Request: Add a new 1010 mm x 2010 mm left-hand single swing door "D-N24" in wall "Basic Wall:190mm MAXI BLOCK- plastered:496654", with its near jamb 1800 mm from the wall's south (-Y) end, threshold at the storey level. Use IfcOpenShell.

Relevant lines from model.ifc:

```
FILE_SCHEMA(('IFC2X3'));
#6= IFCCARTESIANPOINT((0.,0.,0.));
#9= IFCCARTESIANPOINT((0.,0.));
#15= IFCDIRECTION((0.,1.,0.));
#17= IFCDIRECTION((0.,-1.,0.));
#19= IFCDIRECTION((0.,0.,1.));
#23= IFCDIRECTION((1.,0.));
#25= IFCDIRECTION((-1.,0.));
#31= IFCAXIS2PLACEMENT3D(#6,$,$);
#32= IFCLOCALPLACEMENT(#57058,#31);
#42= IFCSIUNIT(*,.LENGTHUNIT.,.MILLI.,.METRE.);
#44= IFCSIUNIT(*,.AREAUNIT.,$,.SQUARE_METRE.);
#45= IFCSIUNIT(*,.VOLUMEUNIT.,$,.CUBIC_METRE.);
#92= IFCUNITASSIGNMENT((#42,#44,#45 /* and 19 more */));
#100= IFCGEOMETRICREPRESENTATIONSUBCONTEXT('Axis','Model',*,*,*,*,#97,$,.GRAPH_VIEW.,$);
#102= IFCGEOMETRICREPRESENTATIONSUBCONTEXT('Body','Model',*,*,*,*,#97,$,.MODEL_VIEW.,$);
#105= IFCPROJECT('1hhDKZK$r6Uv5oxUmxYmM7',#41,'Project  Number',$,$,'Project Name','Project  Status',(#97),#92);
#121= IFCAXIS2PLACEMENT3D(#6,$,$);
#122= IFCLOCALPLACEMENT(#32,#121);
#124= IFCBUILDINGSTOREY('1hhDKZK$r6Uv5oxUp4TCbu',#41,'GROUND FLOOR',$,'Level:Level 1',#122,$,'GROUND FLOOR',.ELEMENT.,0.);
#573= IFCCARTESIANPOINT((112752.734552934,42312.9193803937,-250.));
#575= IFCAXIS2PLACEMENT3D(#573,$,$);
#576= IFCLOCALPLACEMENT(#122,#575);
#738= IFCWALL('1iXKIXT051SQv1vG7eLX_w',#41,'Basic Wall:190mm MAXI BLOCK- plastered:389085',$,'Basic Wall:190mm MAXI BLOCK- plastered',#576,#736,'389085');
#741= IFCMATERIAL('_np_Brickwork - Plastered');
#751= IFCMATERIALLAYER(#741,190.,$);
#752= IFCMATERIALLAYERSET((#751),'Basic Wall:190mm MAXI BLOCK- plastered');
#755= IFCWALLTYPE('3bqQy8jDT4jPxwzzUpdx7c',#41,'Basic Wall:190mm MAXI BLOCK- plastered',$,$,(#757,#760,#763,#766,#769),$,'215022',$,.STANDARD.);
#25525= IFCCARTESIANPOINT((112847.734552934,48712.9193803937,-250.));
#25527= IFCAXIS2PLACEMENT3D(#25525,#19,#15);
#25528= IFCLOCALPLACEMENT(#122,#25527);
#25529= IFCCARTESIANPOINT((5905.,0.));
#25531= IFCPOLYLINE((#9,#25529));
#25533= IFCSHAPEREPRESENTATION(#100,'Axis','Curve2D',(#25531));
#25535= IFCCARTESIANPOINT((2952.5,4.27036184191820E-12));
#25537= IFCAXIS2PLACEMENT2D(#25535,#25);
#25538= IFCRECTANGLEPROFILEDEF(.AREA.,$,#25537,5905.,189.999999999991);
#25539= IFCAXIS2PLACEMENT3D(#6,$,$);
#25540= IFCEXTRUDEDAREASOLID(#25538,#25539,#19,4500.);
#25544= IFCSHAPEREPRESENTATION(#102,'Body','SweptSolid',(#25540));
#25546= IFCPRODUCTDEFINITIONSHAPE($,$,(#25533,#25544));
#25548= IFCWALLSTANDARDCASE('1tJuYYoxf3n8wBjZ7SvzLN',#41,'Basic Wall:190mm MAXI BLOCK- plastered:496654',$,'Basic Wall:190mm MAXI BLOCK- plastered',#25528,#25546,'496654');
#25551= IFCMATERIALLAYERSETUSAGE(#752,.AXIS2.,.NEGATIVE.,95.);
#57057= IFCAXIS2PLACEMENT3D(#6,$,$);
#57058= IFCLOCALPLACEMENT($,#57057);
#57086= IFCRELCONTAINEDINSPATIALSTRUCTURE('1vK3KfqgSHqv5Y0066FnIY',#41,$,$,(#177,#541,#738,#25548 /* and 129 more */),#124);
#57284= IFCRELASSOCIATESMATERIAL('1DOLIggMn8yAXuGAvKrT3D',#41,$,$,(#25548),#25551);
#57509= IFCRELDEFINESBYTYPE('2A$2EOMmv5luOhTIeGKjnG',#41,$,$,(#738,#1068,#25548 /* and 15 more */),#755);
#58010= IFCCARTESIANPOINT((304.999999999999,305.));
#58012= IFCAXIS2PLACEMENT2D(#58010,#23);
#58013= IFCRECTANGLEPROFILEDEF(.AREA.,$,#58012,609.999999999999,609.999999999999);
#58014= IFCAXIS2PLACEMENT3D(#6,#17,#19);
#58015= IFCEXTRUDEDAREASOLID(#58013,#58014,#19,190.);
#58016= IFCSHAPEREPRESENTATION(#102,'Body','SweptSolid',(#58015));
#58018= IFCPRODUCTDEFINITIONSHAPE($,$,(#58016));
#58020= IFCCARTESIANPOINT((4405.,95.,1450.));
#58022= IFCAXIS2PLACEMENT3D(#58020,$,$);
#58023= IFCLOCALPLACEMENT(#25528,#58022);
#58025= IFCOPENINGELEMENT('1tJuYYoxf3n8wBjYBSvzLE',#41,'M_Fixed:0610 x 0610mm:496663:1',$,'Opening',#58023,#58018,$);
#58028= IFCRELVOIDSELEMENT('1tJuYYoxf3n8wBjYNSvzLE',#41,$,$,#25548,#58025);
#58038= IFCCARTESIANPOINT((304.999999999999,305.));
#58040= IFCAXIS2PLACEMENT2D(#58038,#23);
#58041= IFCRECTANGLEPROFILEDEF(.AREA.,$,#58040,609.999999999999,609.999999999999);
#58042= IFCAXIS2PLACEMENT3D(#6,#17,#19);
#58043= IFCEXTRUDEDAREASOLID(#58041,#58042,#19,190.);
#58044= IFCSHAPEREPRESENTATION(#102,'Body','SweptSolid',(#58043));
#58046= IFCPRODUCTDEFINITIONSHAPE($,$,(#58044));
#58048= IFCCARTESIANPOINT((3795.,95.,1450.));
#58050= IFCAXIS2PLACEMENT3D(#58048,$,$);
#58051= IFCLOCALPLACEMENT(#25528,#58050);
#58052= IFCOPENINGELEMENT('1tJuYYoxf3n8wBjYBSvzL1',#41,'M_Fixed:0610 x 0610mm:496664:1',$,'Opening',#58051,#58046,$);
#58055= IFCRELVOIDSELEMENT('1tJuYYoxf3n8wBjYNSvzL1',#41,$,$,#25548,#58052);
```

```python
import numpy as np
import ifcopenshell
import ifcopenshell.api.feature
import ifcopenshell.api.geometry
import ifcopenshell.api.root
import ifcopenshell.api.spatial
import ifcopenshell.api.type
import ifcopenshell.geom
import ifcopenshell.util.element
import ifcopenshell.util.placement
import ifcopenshell.util.representation
import ifcopenshell.util.shape
import ifcopenshell.util.unit

model = ifcopenshell.open("model.ifc")
unit_scale = ifcopenshell.util.unit.calculate_unit_scale(model)
settings = ifcopenshell.geom.settings()


def volume(element):
    """Net volume in cubic metres, openings subtracted."""
    shape = ifcopenshell.geom.create_shape(settings, element)
    return ifcopenshell.util.shape.get_volume(shape.geometry)


wall = model.by_guid("1tJuYYoxf3n8wBjZ7SvzLN")
storey = ifcopenshell.util.element.get_container(wall, ifc_class="IfcBuildingStorey")
context = ifcopenshell.util.representation.get_context(model, "Model", "Body", "MODEL_VIEW")
before = volume(wall)

width, height, from_end, sill = 1.01, 2.01, 1.8, 0.0  # metres

# The wall runs along its own X axis, and the end named is its -X end.
wall_shape = ifcopenshell.geom.create_shape(settings, wall)
x, y, z = ifcopenshell.util.shape.get_vertices(wall_shape.geometry).T
start = x.min() + from_end
face, thickness = float(y.min()), float(y.max() - y.min())
wall_matrix = ifcopenshell.util.placement.get_local_placement(wall.ObjectPlacement)
level = ifcopenshell.util.placement.get_local_placement(storey.ObjectPlacement)[2, 3]


def in_wall(x, y):
    """Placement at x, y metres in the wall's axes, at sill height."""
    matrix = wall_matrix.copy()
    matrix[:, 3] = wall_matrix @ np.array([x / unit_scale, y / unit_scale, 0.0, 1.0])
    matrix[2, 3] = level + sill / unit_scale
    return matrix


# Opening: a box that overshoots both wall faces by 50 mm.
opening = ifcopenshell.api.root.create_entity(model, ifc_class="IfcOpeningElement")
box = ifcopenshell.api.geometry.add_wall_representation(
    model, context=context, length=width, height=height, thickness=thickness + 0.1
)
ifcopenshell.api.geometry.assign_representation(model, product=opening, representation=box)
ifcopenshell.api.geometry.edit_object_placement(model, product=opening, matrix=in_wall(start, face - 0.05), is_si=False)
ifcopenshell.api.feature.add_feature(model, feature=opening, element=wall)

door = ifcopenshell.api.root.create_entity(model, ifc_class="IfcDoor", name="D-N24")
door.OverallWidth, door.OverallHeight = width / unit_scale, height / unit_scale
body = ifcopenshell.api.geometry.add_door_representation(
    model,
    context=context,
    overall_width=door.OverallWidth,
    overall_height=door.OverallHeight,
    operation_type="SINGLE_SWING_LEFT",
    lining_properties={"LiningDepth": thickness / unit_scale, "ThresholdDepth": thickness / unit_scale},
)
ifcopenshell.api.geometry.assign_representation(model, product=door, representation=body)
ifcopenshell.api.spatial.assign_container(model, products=[door], relating_structure=storey)
fills = ifcopenshell.api.feature.add_filling(model, opening=opening, element=door)
fills.OwnerHistory = door.OwnerHistory  # required in IFC2X3

# IFC2X3 keeps the operation on the door style.
style = ifcopenshell.api.root.create_entity(model, ifc_class="IfcDoorStyle", name="D-N24")
style.OperationType, style.ConstructionType = "SINGLE_SWING_LEFT", "NOTDEFINED"
style.ParameterTakesPrecedence = style.Sizeable = False
ifcopenshell.api.type.assign_type(model, related_objects=[door], relating_type=style)

# The lining spans the wall, so the door starts at the wall face.
ifcopenshell.api.geometry.edit_object_placement(model, product=door, matrix=in_wall(start, face), is_si=False)

after = volume(wall)

print(f"wall volume {before:.3f} -> {after:.3f} m3")

model.write("model-out.ifc")
```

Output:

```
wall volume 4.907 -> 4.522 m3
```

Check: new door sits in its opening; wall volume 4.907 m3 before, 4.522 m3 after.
